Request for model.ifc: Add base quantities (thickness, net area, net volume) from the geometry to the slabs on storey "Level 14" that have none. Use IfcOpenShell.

First a look at what the model holds.

```python
import ifcopenshell
import ifcopenshell.util.element
import ifcopenshell.util.unit

model = ifcopenshell.open("model.ifc")
print(model.schema)
for unit_type in ("LENGTHUNIT", "AREAUNIT", "VOLUMEUNIT"):
    print(unit_type, ifcopenshell.util.unit.calculate_unit_scale(model, unit_type))
storey = next(s for s in model.by_type("IfcBuildingStorey") if s.Name == "Level 14")
slabs = [e for e in ifcopenshell.util.element.get_decomposition(storey) if e.is_a("IfcSlab")]
for e in sorted(slabs, key=lambda e: e.id()):
    print(e.id(), e.is_a(), e.Name, list(ifcopenshell.util.element.get_psets(e, qtos_only=True)), sep=" | ")
```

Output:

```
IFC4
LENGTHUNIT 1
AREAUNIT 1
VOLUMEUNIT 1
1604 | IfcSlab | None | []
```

```python
import ifcopenshell
import ifcopenshell.api.pset
import ifcopenshell.geom
import ifcopenshell.util.element
import ifcopenshell.util.shape
import ifcopenshell.util.unit

model = ifcopenshell.open("model.ifc")
unit_scale = ifcopenshell.util.unit.calculate_unit_scale(model)
area_scale = ifcopenshell.util.unit.calculate_unit_scale(model, "AREAUNIT")
volume_scale = ifcopenshell.util.unit.calculate_unit_scale(model, "VOLUMEUNIT")
settings = ifcopenshell.geom.settings()

storey = next(s for s in model.by_type("IfcBuildingStorey") if s.Name == "Level 14")
slabs = [e for e in ifcopenshell.util.element.get_decomposition(storey) if e.is_a("IfcSlab")]

for e in sorted(slabs, key=lambda e: e.id()):
    if ifcopenshell.util.element.get_psets(e, qtos_only=True, should_inherit=False):
        continue
    # Geometry comes back in metres, in the element's own axes.
    shape = ifcopenshell.geom.create_shape(settings, e)
    values = {
        "Width": ifcopenshell.util.shape.get_z(shape.geometry) / unit_scale,
        "NetArea": ifcopenshell.util.shape.get_footprint_area(shape.geometry) / area_scale,
        "NetVolume": ifcopenshell.util.shape.get_volume(shape.geometry) / volume_scale,
    }
    qto = ifcopenshell.api.pset.add_qto(model, product=e, name="Qto_SlabBaseQuantities")
    ifcopenshell.api.pset.edit_qto(model, qto=qto, properties=values)
    print(e.id(), {k: round(v, 3) for k, v in values.items()})

model.write("model_v2.ifc")
```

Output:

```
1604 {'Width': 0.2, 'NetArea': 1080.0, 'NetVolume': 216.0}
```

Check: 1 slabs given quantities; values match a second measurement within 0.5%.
